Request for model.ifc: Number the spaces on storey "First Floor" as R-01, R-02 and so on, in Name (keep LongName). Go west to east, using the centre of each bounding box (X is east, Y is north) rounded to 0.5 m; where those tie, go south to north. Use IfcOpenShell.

First a look at what the model holds.

```python
import ifcopenshell
import ifcopenshell.util.element
import ifcopenshell.util.placement

model = ifcopenshell.open("model.ifc")
print(model.schema)
storey = next(s for s in model.by_type("IfcBuildingStorey") if s.Name == "First Floor")
spaces = [e for e in ifcopenshell.util.element.get_decomposition(storey) if e.is_a("IfcSpace")]
for e in sorted(spaces, key=lambda e: e.id()):
    origin = ifcopenshell.util.placement.get_local_placement(e.ObjectPlacement)[:3, 3]
    print(e.id(), e.Name, e.LongName, origin.round(2) + 0.0, sep=" | ")
```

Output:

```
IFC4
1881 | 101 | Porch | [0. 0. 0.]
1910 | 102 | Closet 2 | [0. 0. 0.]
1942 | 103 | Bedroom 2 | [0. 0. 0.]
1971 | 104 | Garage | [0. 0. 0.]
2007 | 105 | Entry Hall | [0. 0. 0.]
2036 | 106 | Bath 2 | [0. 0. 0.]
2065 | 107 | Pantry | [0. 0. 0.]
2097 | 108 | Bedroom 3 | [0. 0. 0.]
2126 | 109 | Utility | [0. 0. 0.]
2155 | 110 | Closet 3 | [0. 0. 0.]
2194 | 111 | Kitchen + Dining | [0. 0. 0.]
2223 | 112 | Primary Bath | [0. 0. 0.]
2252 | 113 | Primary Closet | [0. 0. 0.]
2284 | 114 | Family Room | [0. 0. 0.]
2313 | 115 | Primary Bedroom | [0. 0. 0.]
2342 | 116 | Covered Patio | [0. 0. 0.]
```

```python
import ifcopenshell
import ifcopenshell.geom
import ifcopenshell.util.element
import ifcopenshell.util.shape

model = ifcopenshell.open("model.ifc")
settings = ifcopenshell.geom.settings()
settings.set("use-world-coords", True)


def centre(element):
    shape = ifcopenshell.geom.create_shape(settings, element)
    return ifcopenshell.util.shape.get_bbox_centroid(shape.geometry)


storey = next(s for s in model.by_type("IfcBuildingStorey") if s.Name == "First Floor")
spaces = [e for e in ifcopenshell.util.element.get_decomposition(storey) if e.is_a("IfcSpace")]

# Insertion points can sit at a corner or the storey origin, so sort by the geometry (in metres).
centres = {e: centre(e) for e in spaces}
spaces.sort(key=lambda e: (round(centres[e][0] / 0.5), centres[e][1]))

for i, e in enumerate(spaces, start=1):
    number = f"R-{i:02d}"
    e.Name = number
    print(e.id(), number)

model.write("model_v2.ifc")
```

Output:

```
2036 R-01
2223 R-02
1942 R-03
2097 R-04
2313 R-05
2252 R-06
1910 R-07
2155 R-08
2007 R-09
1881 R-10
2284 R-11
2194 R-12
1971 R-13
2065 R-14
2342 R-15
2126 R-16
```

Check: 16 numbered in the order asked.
